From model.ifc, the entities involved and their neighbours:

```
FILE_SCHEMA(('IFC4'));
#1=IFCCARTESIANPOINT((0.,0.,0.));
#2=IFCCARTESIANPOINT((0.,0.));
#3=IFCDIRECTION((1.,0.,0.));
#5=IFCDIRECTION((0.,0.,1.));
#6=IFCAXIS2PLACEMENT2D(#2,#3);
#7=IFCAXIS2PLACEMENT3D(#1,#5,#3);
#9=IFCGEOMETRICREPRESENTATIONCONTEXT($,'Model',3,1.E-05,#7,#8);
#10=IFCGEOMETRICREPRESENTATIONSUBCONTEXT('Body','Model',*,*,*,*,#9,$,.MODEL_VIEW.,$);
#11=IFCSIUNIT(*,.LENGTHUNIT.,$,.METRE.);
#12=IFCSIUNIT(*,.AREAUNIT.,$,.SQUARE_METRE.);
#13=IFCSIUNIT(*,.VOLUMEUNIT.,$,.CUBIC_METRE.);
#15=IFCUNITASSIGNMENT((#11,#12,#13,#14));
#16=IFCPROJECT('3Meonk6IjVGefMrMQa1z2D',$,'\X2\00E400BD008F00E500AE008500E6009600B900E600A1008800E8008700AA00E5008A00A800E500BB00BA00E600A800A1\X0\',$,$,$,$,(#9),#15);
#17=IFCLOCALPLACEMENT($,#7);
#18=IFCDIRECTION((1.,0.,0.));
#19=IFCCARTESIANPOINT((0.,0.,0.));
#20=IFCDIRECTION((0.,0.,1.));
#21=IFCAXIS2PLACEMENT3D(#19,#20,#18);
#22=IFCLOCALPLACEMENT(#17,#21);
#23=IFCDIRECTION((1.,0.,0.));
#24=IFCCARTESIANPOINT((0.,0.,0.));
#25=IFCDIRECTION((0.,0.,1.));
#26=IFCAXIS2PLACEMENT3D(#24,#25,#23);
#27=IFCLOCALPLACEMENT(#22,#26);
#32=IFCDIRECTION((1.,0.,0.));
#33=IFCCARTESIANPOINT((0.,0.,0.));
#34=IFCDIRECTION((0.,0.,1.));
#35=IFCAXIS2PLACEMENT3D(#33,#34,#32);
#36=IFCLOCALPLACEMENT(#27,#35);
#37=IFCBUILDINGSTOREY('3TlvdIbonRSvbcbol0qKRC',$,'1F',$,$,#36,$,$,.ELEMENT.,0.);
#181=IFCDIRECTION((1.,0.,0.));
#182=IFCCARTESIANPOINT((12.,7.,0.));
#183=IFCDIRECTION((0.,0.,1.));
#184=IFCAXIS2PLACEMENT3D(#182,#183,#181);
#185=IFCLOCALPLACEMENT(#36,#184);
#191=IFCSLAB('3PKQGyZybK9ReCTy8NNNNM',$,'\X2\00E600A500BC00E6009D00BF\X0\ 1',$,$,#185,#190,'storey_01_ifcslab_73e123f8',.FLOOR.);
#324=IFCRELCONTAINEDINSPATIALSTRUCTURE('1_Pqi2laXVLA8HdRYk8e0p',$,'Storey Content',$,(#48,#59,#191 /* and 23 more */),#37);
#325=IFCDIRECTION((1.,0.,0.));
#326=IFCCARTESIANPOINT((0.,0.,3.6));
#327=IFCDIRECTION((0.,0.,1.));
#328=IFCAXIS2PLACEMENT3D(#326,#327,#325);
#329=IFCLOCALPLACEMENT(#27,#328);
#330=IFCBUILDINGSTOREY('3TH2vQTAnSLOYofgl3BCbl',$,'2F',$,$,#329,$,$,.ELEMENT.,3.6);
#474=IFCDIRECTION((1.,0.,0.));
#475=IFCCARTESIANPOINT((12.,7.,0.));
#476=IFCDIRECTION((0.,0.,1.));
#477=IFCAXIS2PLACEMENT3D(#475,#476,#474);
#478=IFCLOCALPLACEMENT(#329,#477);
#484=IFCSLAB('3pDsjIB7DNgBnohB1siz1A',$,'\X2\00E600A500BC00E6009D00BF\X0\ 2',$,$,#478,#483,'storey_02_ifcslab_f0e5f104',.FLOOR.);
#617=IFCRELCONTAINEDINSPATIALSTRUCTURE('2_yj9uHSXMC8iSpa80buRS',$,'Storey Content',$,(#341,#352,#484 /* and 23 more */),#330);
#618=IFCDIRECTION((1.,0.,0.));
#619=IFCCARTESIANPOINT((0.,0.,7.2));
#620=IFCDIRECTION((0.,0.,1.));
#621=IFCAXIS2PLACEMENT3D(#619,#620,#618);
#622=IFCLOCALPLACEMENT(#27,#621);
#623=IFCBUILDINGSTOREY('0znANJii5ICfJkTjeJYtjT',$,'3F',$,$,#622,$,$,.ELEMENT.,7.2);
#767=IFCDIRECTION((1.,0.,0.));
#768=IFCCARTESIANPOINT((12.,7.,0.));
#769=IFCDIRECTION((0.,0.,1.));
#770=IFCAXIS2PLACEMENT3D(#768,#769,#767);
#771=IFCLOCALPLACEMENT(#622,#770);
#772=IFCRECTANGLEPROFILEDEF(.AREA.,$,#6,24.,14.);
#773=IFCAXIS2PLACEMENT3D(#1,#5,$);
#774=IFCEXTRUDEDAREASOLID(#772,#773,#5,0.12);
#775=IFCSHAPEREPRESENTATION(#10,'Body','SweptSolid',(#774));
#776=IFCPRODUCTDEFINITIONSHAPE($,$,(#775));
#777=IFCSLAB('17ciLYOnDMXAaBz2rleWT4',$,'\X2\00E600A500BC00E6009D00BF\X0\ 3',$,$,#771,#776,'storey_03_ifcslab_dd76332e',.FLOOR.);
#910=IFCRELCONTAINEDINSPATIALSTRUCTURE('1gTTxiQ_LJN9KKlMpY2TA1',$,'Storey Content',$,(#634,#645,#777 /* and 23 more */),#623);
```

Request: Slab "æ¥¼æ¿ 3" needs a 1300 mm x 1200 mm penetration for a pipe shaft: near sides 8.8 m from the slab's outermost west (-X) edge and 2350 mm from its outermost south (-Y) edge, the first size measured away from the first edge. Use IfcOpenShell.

```python
import numpy as np
import ifcopenshell
import ifcopenshell.api.feature
import ifcopenshell.api.geometry
import ifcopenshell.api.root
import ifcopenshell.geom
import ifcopenshell.util.placement
import ifcopenshell.util.representation
import ifcopenshell.util.shape
import ifcopenshell.util.unit

model = ifcopenshell.open("model.ifc")
unit_scale = ifcopenshell.util.unit.calculate_unit_scale(model)
settings = ifcopenshell.geom.settings()


def volume(element):
    """Net volume in cubic metres, openings subtracted."""
    shape = ifcopenshell.geom.create_shape(settings, element)
    return ifcopenshell.util.shape.get_volume(shape.geometry)


slab = model.by_guid("17ciLYOnDMXAaBz2rleWT4")
before = volume(slab)

# Extent in the slab's own axes, in metres. The edges named are its -X and -Y sides.
slab_shape = ifcopenshell.geom.create_shape(settings, slab)
vertices = ifcopenshell.util.shape.get_vertices(slab_shape.geometry)
x_min, y_min, bottom = vertices.min(axis=0)
top = vertices[:, 2].max()

opening = ifcopenshell.api.root.create_entity(model, ifc_class="IfcOpeningElement", name="Pipe shaft opening", predefined_type="OPENING")
context = ifcopenshell.util.representation.get_context(model, "Model", "Body", "MODEL_VIEW")
width, depth = 1.3, 1.2
outline = [(0.0, 0.0), (width, 0.0), (width, depth), (0.0, depth), (0.0, 0.0)]
# Overshoot both faces by 50 mm so the cut is clean.
shape = ifcopenshell.api.geometry.add_slab_representation(
    model, context=context, depth=top - bottom + 0.1, polyline=outline
)
ifcopenshell.api.geometry.assign_representation(model, product=opening, representation=shape)

matrix = ifcopenshell.util.placement.get_local_placement(slab.ObjectPlacement)
matrix[:, 3] = matrix @ np.append(np.array([x_min + 8.8, y_min + 2.35, bottom - 0.05]) / unit_scale, 1.0)
ifcopenshell.api.geometry.edit_object_placement(model, product=opening, matrix=matrix, is_si=False)
ifcopenshell.api.feature.add_feature(model, feature=opening, element=slab)

after = volume(slab)

print(f"slab volume {before:.3f} -> {after:.3f} m3")

model.write("model-out.ifc")
```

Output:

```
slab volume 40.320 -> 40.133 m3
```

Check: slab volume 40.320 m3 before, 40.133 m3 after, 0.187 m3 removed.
